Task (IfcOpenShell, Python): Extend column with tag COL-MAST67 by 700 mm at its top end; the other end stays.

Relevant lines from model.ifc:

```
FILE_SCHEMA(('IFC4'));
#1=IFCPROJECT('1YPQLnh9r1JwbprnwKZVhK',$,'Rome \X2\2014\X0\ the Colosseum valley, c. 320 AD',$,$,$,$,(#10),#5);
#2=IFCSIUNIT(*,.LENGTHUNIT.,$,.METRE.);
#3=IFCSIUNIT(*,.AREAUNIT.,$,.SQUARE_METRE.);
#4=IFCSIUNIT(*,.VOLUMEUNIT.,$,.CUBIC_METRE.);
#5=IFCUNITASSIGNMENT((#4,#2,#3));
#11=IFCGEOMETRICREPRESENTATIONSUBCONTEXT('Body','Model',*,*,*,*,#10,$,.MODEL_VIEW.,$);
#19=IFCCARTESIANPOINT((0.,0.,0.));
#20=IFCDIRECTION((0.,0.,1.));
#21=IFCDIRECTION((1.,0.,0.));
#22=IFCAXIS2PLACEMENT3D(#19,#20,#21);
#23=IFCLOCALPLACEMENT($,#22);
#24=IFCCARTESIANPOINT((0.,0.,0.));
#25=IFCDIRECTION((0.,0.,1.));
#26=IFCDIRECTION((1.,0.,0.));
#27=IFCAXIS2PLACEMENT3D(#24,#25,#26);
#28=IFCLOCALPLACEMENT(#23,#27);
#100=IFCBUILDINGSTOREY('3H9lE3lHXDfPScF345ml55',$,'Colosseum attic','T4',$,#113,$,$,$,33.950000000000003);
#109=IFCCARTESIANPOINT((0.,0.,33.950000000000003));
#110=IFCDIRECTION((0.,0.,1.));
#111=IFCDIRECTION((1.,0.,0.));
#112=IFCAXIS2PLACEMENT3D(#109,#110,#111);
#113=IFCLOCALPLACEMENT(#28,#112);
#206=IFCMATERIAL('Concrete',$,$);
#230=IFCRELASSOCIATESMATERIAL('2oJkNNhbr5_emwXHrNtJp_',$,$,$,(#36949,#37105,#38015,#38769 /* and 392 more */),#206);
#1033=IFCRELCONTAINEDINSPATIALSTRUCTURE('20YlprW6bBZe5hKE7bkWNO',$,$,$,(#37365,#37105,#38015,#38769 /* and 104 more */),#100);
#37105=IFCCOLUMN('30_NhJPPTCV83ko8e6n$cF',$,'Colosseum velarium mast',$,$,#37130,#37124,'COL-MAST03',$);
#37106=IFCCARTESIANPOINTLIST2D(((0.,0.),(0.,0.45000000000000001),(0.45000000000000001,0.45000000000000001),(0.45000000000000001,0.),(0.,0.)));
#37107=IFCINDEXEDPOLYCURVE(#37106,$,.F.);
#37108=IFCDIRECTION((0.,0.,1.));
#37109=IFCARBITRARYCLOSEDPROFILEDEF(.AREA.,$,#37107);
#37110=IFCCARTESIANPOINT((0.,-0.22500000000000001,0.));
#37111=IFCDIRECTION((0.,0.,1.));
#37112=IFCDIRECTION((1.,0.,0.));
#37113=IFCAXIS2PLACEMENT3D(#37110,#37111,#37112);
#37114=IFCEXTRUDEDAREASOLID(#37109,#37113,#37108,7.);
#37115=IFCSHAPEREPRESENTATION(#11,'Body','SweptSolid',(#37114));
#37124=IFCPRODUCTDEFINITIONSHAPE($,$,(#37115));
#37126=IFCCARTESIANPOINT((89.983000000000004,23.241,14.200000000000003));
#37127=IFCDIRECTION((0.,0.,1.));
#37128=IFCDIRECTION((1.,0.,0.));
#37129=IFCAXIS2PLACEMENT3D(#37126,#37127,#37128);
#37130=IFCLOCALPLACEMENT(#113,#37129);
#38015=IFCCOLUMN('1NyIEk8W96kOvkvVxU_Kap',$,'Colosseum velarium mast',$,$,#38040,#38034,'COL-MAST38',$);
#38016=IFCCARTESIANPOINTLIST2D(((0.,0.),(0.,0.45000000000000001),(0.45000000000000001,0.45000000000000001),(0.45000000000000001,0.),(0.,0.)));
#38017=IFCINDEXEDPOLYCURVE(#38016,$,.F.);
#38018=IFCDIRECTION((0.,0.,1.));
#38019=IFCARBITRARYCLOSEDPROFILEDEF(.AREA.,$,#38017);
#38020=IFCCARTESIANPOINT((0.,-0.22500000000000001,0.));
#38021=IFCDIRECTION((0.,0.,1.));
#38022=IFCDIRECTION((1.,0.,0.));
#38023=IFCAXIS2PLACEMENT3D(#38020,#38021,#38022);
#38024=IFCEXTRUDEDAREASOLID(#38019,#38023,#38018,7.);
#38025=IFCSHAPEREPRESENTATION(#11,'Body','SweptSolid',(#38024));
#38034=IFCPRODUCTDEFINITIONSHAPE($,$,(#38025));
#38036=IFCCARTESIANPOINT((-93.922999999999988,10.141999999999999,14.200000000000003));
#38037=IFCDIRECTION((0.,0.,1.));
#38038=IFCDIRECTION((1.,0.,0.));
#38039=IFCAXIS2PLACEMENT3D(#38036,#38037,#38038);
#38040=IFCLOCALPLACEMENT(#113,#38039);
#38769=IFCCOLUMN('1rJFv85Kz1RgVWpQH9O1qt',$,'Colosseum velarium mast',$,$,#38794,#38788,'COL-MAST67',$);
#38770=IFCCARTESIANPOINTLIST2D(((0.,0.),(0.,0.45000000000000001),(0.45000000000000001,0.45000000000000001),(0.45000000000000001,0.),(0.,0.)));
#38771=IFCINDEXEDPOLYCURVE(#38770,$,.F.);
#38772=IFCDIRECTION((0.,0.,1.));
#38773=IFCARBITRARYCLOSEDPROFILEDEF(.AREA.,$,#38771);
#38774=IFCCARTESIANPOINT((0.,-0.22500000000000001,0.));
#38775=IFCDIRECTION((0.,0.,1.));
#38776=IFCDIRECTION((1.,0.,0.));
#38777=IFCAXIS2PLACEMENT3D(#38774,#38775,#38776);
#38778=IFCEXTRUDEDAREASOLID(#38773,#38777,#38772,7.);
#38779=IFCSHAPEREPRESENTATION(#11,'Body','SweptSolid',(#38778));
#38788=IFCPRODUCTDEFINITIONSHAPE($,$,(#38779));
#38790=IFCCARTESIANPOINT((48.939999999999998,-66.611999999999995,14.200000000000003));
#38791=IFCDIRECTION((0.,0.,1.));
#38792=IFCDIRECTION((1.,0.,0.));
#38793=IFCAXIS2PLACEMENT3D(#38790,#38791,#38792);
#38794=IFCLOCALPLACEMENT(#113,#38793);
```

```python
import ifcopenshell
import ifcopenshell.util.representation

model = ifcopenshell.open("model.ifc")

member = model.by_guid("1rJFv85Kz1RgVWpQH9O1qt")
change = 0.7

# The extrusion runs towards the end named, so only its depth changes.
body = ifcopenshell.util.representation.get_representation(member, "Model", "Body")
solid = body.Items[0]
old_length = solid.Depth
solid.Depth += change

print(f"length {old_length:g} -> {solid.Depth:g}")

model.write("model_rev.ifc")
```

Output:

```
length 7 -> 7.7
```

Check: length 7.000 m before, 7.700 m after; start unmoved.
